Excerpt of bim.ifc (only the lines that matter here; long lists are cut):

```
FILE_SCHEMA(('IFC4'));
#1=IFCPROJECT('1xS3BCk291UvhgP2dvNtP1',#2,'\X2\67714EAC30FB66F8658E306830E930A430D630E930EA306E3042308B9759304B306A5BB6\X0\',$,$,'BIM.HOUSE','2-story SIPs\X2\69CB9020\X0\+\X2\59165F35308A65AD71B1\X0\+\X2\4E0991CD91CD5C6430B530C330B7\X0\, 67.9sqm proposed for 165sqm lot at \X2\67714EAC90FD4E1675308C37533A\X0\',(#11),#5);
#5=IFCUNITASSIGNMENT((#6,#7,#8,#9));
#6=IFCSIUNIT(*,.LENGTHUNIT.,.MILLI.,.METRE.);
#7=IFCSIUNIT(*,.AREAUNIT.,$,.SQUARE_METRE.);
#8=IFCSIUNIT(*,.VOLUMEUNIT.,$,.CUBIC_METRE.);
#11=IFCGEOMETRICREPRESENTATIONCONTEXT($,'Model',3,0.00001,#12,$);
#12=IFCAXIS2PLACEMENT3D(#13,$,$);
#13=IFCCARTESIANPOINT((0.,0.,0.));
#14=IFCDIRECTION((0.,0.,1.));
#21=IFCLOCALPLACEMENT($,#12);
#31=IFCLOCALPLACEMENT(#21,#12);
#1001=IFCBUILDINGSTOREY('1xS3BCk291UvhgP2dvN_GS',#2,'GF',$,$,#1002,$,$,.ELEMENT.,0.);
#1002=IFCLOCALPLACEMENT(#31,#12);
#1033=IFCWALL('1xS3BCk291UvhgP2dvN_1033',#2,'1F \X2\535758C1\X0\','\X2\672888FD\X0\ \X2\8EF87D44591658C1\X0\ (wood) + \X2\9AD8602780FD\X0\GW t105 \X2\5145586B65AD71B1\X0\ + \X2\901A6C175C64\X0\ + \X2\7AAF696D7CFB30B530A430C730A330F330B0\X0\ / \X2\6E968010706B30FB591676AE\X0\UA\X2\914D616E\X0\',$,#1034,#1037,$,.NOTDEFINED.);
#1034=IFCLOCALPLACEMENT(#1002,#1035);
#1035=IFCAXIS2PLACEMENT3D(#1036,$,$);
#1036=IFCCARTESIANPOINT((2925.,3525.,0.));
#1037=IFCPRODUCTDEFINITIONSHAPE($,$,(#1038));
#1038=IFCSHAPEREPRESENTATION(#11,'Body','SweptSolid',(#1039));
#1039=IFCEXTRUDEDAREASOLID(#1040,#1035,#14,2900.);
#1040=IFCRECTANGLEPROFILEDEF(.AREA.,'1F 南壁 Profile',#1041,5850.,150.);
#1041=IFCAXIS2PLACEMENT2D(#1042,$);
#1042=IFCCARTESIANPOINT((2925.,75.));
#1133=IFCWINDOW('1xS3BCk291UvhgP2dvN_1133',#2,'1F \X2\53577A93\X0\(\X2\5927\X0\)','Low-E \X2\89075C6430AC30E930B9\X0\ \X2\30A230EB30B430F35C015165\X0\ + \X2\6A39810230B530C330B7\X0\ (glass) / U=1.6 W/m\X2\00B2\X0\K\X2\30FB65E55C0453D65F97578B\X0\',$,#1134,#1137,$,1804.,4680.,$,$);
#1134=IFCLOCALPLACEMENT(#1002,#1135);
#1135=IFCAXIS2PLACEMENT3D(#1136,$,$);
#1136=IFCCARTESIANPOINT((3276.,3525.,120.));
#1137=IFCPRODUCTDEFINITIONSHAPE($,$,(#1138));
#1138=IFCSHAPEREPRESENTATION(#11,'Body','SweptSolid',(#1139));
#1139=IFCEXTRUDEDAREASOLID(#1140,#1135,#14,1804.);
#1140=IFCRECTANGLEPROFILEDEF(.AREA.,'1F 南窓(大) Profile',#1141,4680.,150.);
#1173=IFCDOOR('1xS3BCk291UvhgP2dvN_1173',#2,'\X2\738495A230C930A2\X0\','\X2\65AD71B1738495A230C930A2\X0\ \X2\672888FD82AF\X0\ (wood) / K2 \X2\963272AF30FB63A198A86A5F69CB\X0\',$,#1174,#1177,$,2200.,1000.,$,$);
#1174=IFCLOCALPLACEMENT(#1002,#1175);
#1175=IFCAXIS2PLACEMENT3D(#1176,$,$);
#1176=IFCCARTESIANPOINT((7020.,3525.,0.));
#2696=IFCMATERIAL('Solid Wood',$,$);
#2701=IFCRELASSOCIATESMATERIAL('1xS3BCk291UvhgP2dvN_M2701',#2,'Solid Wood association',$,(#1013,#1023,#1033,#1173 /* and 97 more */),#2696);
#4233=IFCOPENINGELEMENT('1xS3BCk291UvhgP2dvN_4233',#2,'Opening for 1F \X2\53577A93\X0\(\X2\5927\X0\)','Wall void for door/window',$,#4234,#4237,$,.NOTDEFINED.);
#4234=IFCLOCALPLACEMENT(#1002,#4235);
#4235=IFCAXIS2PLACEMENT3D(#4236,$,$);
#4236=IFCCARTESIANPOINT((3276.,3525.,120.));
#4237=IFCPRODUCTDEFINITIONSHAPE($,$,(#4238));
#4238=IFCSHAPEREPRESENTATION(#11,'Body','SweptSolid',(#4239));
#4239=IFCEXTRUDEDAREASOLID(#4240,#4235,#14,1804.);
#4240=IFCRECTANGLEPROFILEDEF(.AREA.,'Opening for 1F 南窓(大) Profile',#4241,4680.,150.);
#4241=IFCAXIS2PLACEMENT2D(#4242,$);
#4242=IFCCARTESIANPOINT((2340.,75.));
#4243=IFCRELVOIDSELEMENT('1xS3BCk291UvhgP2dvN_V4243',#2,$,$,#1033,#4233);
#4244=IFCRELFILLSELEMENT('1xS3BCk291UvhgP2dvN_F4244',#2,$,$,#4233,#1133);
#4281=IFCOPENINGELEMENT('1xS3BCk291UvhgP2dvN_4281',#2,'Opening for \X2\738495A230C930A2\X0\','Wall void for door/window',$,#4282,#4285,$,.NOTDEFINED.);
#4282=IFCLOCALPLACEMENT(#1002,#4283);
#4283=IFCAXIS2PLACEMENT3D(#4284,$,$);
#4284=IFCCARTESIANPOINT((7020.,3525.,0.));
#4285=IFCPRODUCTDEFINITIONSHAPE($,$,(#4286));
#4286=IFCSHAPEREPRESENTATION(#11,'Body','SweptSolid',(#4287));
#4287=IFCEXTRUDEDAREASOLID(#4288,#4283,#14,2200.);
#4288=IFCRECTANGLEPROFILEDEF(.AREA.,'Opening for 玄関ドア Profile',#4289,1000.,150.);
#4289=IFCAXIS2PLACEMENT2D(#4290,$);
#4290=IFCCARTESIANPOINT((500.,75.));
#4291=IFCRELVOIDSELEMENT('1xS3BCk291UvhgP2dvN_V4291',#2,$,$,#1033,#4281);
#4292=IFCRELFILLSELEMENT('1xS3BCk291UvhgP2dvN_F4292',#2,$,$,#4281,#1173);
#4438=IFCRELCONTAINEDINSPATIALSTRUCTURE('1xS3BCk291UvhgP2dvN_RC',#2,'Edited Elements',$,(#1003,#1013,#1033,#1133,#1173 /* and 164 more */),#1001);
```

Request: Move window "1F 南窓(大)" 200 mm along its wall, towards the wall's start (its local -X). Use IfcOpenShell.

```python
import ifcopenshell
import ifcopenshell.api.geometry
import ifcopenshell.util.placement

model = ifcopenshell.open("bim.ifc")

window = model.by_id(1133)
opening = window.FillsVoids[0].RelatingOpeningElement
wall = opening.VoidsElements[0].RelatingBuildingElement

wall_matrix = ifcopenshell.util.placement.get_local_placement(wall.ObjectPlacement)
shift = wall_matrix[:3, 0] * -200.0
before = ifcopenshell.util.placement.get_local_placement(window.ObjectPlacement)[:3, 3].copy()

# The window is not placed relative to its opening, so move both.
for product in (opening, window):
    matrix = ifcopenshell.util.placement.get_local_placement(product.ObjectPlacement)
    matrix[:3, 3] += shift
    ifcopenshell.api.geometry.edit_object_placement(model, product=product, matrix=matrix, is_si=False)

after = ifcopenshell.util.placement.get_local_placement(window.ObjectPlacement)[:3, 3]
print("window moved by", (after - before).round(3) + 0.0)

model.write("bim-out.ifc")
```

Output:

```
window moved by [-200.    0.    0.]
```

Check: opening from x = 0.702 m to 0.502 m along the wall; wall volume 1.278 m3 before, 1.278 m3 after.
